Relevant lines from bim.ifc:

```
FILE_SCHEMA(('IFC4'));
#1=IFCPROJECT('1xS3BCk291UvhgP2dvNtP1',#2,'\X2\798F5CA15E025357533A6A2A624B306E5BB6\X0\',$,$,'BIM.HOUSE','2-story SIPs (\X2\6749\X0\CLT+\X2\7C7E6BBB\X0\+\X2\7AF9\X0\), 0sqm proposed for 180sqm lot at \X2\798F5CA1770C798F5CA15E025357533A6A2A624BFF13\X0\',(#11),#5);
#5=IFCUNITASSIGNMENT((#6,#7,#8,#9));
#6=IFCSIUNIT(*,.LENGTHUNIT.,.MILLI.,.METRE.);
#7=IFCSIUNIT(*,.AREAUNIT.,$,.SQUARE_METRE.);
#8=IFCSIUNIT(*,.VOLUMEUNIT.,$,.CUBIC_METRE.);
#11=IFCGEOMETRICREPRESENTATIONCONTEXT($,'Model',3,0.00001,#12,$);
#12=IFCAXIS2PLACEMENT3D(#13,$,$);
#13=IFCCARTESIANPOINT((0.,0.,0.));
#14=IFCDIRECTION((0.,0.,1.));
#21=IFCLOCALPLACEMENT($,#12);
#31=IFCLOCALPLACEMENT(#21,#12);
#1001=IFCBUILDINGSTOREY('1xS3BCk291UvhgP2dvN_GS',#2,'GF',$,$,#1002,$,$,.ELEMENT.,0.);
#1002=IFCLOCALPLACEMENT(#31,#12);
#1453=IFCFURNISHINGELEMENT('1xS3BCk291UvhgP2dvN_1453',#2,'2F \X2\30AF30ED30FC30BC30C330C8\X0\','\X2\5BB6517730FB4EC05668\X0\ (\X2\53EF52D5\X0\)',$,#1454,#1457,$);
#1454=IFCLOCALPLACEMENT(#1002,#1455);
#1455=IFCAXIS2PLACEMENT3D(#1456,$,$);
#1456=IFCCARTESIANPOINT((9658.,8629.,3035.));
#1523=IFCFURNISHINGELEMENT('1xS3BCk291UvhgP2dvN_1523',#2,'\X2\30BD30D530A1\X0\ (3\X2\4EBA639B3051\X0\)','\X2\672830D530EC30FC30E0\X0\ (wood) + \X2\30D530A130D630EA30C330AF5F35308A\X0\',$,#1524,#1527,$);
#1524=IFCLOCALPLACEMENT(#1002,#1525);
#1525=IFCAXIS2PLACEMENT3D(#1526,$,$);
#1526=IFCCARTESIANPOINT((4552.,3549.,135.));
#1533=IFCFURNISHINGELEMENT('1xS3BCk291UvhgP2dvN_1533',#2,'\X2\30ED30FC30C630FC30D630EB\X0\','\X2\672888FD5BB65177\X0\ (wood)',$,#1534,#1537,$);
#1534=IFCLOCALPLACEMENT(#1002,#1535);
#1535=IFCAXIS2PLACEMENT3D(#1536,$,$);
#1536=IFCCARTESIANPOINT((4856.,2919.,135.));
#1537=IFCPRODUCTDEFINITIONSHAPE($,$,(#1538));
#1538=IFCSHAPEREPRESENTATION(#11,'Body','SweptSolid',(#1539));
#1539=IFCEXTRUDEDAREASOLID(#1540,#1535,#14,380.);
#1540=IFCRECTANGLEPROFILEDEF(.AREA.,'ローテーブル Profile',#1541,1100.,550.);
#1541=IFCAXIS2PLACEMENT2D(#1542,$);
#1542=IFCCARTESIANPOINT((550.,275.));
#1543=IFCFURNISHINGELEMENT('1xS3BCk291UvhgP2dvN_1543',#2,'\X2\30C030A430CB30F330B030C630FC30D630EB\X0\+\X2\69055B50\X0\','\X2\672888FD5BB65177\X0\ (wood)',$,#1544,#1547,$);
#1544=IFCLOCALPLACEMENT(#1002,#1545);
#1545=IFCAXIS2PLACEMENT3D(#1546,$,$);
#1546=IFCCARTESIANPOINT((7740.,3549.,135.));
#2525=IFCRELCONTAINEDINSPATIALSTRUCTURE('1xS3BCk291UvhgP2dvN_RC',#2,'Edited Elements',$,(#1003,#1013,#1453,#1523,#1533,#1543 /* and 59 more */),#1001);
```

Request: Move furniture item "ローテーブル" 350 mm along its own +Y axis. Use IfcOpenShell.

```python
import ifcopenshell
import ifcopenshell.api.geometry
import ifcopenshell.util.placement

model = ifcopenshell.open("bim.ifc")

item = model.by_id(1533)
matrix = ifcopenshell.util.placement.get_local_placement(item.ObjectPlacement)
matrix[:3, 3] += matrix[:3, 1] * 350.0
ifcopenshell.api.geometry.edit_object_placement(model, product=item, matrix=matrix, is_si=False)

print(ifcopenshell.util.placement.get_local_placement(item.ObjectPlacement).round(3) + 0.0)

model.write("bim_edited.ifc")
```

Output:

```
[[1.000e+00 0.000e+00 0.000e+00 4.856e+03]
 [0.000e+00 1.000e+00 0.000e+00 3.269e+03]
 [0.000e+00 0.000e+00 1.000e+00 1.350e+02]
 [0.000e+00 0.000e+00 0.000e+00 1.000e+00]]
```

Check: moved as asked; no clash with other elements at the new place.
